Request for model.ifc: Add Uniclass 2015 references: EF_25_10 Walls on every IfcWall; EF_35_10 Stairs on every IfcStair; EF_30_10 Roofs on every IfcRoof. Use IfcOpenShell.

First a look at what the model holds.

```python
import ifcopenshell

model = ifcopenshell.open("model.ifc")
print(model.schema)
print("classifications:", [c.Name for c in model.by_type("IfcClassification")])
for ifc_class in ("IfcDoor", "IfcRoof", "IfcStair", "IfcWall", "IfcWindow"):
    print(ifc_class, len(model.by_type(ifc_class)))
```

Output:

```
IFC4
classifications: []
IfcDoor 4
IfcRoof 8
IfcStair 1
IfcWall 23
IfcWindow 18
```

```python
import ifcopenshell
import ifcopenshell.api.classification

model = ifcopenshell.open("model.ifc")

system = ifcopenshell.api.classification.add_classification(model, classification="Uniclass 2015")

codes = {
    "IfcWall": ("EF_25_10", "Walls"),
    "IfcStair": ("EF_35_10", "Stairs"),
    "IfcRoof": ("EF_30_10", "Roofs"),
}
for ifc_class, (code, name) in codes.items():
    products = model.by_type(ifc_class)
    ifcopenshell.api.classification.add_reference(
        model, products=products, classification=system, identification=code, name=name
    )
    print(code, len(products))

model.write("model_v2.ifc")
```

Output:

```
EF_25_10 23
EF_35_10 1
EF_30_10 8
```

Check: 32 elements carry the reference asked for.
